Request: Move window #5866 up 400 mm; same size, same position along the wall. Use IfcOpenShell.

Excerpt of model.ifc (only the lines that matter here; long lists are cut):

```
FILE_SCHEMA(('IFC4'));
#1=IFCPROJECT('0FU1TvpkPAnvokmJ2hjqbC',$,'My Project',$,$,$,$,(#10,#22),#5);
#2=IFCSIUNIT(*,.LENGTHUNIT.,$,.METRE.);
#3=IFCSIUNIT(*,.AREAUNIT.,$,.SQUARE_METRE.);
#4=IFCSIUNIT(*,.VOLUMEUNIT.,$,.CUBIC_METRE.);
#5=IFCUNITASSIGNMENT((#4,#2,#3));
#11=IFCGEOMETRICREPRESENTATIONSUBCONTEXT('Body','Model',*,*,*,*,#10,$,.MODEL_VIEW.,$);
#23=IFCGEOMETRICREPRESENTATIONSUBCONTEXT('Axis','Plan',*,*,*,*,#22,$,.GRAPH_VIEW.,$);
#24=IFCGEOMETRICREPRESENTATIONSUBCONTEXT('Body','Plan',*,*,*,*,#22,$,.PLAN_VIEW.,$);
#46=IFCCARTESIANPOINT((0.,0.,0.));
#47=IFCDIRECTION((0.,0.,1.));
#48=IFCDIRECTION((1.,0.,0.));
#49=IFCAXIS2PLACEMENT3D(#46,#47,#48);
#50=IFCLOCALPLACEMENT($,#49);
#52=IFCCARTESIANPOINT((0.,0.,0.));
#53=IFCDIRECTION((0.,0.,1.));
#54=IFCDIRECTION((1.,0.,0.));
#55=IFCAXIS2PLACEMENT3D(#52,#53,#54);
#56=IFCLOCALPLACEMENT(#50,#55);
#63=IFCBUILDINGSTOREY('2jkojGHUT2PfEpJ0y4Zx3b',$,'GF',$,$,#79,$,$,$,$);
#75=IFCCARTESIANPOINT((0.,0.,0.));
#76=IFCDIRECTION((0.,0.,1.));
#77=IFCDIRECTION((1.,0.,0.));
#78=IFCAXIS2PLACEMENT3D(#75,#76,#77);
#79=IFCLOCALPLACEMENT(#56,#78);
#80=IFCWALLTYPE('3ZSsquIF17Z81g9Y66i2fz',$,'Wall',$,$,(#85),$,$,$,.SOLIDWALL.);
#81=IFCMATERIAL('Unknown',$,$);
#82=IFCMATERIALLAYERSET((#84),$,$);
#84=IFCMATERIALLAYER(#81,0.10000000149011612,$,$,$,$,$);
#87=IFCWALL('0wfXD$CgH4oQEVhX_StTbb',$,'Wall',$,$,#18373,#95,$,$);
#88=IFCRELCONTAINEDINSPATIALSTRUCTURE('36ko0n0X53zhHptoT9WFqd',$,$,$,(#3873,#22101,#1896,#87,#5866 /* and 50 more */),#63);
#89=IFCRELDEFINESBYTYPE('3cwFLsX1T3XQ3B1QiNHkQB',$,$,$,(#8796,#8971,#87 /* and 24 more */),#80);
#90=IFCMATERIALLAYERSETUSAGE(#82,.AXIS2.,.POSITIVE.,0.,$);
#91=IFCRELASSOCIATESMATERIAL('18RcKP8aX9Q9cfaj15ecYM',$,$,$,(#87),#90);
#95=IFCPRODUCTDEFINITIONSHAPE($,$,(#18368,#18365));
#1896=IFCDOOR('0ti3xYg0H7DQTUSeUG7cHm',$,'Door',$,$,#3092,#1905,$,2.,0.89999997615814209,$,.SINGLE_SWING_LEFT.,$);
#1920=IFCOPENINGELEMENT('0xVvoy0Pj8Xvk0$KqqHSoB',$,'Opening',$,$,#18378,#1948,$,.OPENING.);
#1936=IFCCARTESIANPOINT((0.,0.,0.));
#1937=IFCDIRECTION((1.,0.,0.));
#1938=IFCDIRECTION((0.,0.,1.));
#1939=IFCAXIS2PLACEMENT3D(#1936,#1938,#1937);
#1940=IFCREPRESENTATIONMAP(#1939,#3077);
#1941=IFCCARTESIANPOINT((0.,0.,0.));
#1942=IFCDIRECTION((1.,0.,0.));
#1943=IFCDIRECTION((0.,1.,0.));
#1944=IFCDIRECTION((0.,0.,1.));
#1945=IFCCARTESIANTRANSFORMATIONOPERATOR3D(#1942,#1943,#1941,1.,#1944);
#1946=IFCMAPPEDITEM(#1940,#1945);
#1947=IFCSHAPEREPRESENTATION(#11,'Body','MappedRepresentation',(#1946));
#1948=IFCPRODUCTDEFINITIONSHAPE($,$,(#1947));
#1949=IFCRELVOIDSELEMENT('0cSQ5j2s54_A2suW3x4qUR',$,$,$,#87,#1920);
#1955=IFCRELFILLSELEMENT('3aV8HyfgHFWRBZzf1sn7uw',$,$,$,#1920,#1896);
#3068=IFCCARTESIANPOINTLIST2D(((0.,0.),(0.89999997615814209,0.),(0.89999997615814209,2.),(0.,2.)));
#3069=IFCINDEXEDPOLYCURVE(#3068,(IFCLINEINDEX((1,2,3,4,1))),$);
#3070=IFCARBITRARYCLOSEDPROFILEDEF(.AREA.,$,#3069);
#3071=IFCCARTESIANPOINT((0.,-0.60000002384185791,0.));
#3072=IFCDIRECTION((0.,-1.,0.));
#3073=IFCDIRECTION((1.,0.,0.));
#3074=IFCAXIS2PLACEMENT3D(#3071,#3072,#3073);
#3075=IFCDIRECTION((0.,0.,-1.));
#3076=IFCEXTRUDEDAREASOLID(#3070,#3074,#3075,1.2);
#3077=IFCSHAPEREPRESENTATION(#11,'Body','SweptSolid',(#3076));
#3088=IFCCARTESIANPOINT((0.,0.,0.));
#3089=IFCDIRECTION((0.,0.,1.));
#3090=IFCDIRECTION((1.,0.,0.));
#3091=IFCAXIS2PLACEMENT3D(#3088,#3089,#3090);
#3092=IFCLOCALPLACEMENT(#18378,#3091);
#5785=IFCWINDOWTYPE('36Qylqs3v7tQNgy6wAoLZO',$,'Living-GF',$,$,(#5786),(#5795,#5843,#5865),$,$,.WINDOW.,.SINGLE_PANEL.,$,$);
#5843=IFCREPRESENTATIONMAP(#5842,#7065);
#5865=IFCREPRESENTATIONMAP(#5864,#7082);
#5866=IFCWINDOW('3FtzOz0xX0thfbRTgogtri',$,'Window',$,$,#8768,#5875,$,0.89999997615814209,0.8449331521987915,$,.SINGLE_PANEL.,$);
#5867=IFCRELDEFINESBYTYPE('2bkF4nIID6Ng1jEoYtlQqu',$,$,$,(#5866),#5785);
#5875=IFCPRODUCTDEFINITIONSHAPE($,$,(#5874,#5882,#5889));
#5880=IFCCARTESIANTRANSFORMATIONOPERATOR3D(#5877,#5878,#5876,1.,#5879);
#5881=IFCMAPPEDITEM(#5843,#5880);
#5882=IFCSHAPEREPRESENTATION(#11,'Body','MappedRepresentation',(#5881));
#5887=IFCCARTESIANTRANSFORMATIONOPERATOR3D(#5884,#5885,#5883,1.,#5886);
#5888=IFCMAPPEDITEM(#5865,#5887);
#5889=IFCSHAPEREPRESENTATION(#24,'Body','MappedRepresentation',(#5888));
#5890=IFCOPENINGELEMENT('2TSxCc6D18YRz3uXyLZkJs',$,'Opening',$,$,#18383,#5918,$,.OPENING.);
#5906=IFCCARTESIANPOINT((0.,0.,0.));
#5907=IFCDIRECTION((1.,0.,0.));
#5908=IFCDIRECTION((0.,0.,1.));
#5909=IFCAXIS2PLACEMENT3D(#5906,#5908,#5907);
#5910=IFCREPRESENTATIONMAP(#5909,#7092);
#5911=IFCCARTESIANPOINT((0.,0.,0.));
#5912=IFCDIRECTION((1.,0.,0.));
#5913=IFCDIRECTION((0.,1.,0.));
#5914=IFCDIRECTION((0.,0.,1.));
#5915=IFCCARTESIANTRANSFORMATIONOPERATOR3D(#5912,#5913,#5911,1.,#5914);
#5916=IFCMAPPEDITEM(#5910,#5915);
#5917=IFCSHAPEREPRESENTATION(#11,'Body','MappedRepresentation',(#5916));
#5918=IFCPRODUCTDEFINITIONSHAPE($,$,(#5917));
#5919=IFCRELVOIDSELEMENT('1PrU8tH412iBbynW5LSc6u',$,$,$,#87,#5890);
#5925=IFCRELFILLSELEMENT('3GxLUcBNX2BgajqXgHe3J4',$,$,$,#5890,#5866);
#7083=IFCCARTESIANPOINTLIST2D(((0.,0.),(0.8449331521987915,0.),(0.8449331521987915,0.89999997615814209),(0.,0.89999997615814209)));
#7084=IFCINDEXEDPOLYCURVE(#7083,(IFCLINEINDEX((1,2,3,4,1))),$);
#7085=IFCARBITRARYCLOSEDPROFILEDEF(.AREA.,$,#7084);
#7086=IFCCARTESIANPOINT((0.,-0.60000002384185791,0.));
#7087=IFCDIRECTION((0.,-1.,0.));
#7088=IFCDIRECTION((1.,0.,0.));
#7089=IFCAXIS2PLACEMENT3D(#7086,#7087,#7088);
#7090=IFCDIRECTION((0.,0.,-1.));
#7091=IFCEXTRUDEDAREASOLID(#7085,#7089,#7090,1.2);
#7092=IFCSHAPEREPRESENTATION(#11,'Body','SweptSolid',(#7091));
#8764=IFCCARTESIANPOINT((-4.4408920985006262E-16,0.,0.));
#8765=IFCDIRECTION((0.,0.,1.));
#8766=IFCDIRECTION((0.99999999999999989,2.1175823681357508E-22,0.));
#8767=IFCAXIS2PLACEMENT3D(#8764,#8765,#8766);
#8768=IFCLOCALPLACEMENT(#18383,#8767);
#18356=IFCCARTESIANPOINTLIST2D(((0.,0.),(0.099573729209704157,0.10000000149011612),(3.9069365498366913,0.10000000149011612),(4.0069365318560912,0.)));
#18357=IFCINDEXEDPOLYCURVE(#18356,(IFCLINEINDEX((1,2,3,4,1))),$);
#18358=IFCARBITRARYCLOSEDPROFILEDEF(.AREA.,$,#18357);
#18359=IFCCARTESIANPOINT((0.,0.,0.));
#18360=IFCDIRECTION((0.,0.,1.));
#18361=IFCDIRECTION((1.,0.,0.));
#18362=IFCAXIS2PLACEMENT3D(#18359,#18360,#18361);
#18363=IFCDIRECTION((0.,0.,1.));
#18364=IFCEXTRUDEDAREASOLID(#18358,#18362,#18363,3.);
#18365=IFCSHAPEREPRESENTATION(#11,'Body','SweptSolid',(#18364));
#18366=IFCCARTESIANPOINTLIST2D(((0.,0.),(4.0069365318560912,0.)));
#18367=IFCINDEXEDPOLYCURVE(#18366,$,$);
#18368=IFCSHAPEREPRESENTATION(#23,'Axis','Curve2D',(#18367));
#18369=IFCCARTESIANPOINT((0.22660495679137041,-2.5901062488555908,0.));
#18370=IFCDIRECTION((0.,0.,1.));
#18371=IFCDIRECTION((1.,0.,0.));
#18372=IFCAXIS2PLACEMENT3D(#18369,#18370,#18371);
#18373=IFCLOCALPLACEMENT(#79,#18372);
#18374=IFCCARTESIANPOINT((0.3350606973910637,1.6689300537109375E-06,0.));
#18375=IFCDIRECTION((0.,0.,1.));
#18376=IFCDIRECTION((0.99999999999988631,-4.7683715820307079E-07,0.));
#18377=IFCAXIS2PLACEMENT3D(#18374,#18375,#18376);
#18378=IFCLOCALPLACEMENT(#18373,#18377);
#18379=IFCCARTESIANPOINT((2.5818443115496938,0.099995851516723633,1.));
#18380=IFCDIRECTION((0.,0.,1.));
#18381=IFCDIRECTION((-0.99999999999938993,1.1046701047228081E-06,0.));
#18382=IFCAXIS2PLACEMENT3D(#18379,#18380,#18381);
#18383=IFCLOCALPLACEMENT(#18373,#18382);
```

```python
import numpy as np
import ifcopenshell
import ifcopenshell.api.geometry
import ifcopenshell.util.placement
import ifcopenshell.util.unit

model = ifcopenshell.open("model.ifc")
unit_scale = ifcopenshell.util.unit.calculate_unit_scale(model)

window = model.by_guid("3FtzOz0xX0thfbRTgogtri")
opening = window.FillsVoids[0].RelatingOpeningElement
dz = 0.4 / unit_scale

shift = np.array([0.0, 0.0, dz])
# The window is placed relative to its opening, so it follows when the opening moves.
matrix = ifcopenshell.util.placement.get_local_placement(opening.ObjectPlacement)
matrix[:3, 3] += shift
ifcopenshell.api.geometry.edit_object_placement(
    model, product=opening, matrix=matrix, is_si=False, should_transform_children=True
)

print(f"moved by {dz * unit_scale:+.3f} m")

model.write("model-out.ifc")
```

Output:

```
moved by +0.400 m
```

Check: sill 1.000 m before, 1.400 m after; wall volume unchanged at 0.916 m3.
